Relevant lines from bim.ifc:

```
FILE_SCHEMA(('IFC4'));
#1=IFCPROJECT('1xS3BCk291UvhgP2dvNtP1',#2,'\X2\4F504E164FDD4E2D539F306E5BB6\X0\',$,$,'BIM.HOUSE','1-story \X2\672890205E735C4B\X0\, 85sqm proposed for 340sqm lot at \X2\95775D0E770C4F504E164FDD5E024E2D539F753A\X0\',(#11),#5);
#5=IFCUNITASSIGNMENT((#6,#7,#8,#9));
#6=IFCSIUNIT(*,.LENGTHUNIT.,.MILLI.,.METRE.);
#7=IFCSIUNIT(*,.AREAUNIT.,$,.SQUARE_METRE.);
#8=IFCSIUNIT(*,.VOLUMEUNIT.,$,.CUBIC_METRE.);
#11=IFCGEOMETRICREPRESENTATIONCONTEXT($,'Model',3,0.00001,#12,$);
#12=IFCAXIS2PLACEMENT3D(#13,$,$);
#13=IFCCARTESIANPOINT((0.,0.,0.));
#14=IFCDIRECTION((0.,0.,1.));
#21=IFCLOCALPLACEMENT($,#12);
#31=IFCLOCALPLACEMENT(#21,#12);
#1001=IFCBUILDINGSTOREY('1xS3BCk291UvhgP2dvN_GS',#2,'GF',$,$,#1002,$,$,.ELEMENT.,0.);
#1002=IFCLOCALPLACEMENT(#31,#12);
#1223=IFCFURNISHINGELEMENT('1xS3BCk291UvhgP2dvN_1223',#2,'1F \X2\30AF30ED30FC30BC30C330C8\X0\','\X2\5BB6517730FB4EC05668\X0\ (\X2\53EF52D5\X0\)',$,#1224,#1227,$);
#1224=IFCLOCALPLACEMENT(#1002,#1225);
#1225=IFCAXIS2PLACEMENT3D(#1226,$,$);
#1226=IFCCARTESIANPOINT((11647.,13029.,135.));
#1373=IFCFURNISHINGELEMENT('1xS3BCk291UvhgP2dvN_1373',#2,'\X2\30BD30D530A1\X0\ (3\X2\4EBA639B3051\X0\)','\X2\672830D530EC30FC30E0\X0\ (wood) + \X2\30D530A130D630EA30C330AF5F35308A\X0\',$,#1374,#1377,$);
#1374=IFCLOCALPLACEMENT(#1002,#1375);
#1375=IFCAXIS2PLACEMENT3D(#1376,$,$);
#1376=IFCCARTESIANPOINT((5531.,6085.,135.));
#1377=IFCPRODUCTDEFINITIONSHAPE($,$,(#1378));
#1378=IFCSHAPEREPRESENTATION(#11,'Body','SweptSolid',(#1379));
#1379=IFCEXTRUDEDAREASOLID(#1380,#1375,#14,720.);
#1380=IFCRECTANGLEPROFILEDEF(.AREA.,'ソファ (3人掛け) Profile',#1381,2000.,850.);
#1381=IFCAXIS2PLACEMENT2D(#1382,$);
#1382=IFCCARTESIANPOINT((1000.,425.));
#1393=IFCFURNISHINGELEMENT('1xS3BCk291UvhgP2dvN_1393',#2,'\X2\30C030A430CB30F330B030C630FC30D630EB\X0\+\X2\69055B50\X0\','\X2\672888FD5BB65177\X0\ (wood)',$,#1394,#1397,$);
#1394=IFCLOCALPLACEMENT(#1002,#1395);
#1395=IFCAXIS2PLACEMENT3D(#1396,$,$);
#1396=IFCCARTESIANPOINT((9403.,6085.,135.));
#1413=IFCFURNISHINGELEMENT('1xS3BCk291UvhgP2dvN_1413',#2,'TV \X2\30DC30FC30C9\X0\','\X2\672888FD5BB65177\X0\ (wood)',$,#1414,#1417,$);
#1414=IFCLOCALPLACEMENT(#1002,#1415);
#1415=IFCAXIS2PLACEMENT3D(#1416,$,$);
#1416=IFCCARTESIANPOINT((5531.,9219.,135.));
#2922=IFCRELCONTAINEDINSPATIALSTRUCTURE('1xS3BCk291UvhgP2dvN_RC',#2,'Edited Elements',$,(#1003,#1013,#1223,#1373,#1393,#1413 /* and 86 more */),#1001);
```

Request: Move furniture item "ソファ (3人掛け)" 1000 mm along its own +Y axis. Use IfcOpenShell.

```python
import ifcopenshell
import ifcopenshell.api.geometry
import ifcopenshell.util.placement

model = ifcopenshell.open("bim.ifc")

item = model.by_guid("1xS3BCk291UvhgP2dvN_1373")
matrix = ifcopenshell.util.placement.get_local_placement(item.ObjectPlacement)
matrix[:3, 3] += matrix[:3, 1] * 1000.0
ifcopenshell.api.geometry.edit_object_placement(model, product=item, matrix=matrix, is_si=False)

print(ifcopenshell.util.placement.get_local_placement(item.ObjectPlacement).round(3) + 0.0)

model.write("bim_rev.ifc")
```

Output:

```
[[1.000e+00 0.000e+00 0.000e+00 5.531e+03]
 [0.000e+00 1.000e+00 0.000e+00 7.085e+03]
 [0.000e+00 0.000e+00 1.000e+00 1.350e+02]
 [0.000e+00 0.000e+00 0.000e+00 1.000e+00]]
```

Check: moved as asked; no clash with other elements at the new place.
